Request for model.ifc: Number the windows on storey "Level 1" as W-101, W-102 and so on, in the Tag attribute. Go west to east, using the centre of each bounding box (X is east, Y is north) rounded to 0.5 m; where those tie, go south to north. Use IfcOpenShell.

First a look at what the model holds.

```python
import ifcopenshell
import ifcopenshell.util.element
import ifcopenshell.util.placement

model = ifcopenshell.open("model.ifc")
print(model.schema)
storey = next(s for s in model.by_type("IfcBuildingStorey") if s.Name == "Level 1")
windows = [e for e in ifcopenshell.util.element.get_decomposition(storey) if e.is_a("IfcWindow")]
for e in sorted(windows, key=lambda e: e.id()):
    origin = ifcopenshell.util.placement.get_local_placement(e.ObjectPlacement)[:3, 3]
    print(e.id(), e.Tag, e.Name, origin.round(2) + 0.0, sep=" | ")
```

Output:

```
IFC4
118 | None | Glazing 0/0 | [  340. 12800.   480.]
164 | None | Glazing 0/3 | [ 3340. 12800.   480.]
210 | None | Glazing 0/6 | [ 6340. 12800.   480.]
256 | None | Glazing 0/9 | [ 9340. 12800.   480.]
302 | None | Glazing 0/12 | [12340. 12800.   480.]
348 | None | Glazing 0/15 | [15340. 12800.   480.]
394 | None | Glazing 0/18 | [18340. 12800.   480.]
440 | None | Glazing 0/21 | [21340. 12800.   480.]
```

```python
import ifcopenshell
import ifcopenshell.geom
import ifcopenshell.util.element
import ifcopenshell.util.shape

model = ifcopenshell.open("model.ifc")
settings = ifcopenshell.geom.settings()
settings.set("use-world-coords", True)


def centre(element):
    shape = ifcopenshell.geom.create_shape(settings, element)
    return ifcopenshell.util.shape.get_bbox_centroid(shape.geometry)


storey = next(s for s in model.by_type("IfcBuildingStorey") if s.Name == "Level 1")
windows = [e for e in ifcopenshell.util.element.get_decomposition(storey) if e.is_a("IfcWindow")]

# Insertion points can sit at a corner or the storey origin, so sort by the geometry (in metres).
centres = {e: centre(e) for e in windows}
windows.sort(key=lambda e: (round(centres[e][0] / 0.5), centres[e][1]))

for i, e in enumerate(windows, start=1):
    number = f"W-1{i:02d}"
    e.Tag = number
    print(e.id(), number)

model.write("model_v2.ifc")
```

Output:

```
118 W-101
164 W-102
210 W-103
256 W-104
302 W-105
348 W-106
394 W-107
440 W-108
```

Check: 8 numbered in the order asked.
